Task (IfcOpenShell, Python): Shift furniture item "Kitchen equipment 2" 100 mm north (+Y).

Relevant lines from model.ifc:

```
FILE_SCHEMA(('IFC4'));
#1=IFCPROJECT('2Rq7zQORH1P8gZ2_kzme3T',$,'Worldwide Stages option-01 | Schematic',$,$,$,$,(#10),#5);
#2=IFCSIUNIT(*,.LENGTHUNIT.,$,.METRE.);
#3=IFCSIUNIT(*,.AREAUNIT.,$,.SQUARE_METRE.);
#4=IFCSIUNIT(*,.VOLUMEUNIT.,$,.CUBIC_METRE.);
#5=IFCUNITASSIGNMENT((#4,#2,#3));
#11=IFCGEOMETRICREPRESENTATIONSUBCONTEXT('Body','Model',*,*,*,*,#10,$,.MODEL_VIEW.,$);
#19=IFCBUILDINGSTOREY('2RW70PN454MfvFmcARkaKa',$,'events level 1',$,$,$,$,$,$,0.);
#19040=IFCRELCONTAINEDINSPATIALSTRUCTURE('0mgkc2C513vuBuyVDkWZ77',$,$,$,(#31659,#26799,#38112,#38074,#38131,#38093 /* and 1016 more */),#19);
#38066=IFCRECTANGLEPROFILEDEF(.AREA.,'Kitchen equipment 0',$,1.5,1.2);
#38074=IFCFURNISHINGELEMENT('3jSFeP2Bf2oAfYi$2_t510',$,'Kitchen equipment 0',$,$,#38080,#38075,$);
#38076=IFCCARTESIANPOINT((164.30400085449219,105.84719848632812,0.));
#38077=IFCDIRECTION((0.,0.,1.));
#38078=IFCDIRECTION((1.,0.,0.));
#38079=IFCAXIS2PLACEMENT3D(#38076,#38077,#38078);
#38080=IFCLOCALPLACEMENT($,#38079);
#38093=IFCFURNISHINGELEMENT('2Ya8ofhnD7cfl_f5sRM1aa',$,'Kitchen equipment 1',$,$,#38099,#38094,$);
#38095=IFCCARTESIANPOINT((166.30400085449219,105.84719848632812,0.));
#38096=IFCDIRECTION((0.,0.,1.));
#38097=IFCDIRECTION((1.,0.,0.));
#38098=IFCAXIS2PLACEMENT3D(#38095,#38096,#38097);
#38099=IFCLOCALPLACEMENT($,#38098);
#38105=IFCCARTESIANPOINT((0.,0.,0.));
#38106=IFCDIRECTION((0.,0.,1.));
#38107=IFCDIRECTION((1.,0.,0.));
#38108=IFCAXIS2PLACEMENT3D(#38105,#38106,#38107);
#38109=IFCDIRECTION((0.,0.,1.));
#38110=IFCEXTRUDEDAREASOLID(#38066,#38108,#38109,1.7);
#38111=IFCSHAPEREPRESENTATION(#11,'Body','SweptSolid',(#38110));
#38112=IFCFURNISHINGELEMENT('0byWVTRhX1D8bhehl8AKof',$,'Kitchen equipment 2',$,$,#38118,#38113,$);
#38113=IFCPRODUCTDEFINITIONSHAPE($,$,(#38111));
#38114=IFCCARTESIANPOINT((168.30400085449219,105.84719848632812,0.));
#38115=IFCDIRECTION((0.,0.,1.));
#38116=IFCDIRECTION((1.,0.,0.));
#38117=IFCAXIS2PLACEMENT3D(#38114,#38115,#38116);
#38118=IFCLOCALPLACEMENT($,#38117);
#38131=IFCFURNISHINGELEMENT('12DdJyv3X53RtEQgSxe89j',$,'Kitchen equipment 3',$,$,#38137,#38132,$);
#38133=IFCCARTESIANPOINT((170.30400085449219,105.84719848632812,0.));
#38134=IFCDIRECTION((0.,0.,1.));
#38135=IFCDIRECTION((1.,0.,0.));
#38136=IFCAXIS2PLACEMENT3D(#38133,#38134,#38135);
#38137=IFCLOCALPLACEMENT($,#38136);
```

```python
import ifcopenshell
import ifcopenshell.api.geometry
import ifcopenshell.util.placement
import ifcopenshell.util.unit

model = ifcopenshell.open("model.ifc")
unit_scale = ifcopenshell.util.unit.calculate_unit_scale(model)

item = model.by_id(38112)
matrix = ifcopenshell.util.placement.get_local_placement(item.ObjectPlacement)
matrix[1, 3] += 0.1 / unit_scale
ifcopenshell.api.geometry.edit_object_placement(model, product=item, matrix=matrix, is_si=False)

print(ifcopenshell.util.placement.get_local_placement(item.ObjectPlacement).round(3) + 0.0)

model.write("model_updated.ifc")
```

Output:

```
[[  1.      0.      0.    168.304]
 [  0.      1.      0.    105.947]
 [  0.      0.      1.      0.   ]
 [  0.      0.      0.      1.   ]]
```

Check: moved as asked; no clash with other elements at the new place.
